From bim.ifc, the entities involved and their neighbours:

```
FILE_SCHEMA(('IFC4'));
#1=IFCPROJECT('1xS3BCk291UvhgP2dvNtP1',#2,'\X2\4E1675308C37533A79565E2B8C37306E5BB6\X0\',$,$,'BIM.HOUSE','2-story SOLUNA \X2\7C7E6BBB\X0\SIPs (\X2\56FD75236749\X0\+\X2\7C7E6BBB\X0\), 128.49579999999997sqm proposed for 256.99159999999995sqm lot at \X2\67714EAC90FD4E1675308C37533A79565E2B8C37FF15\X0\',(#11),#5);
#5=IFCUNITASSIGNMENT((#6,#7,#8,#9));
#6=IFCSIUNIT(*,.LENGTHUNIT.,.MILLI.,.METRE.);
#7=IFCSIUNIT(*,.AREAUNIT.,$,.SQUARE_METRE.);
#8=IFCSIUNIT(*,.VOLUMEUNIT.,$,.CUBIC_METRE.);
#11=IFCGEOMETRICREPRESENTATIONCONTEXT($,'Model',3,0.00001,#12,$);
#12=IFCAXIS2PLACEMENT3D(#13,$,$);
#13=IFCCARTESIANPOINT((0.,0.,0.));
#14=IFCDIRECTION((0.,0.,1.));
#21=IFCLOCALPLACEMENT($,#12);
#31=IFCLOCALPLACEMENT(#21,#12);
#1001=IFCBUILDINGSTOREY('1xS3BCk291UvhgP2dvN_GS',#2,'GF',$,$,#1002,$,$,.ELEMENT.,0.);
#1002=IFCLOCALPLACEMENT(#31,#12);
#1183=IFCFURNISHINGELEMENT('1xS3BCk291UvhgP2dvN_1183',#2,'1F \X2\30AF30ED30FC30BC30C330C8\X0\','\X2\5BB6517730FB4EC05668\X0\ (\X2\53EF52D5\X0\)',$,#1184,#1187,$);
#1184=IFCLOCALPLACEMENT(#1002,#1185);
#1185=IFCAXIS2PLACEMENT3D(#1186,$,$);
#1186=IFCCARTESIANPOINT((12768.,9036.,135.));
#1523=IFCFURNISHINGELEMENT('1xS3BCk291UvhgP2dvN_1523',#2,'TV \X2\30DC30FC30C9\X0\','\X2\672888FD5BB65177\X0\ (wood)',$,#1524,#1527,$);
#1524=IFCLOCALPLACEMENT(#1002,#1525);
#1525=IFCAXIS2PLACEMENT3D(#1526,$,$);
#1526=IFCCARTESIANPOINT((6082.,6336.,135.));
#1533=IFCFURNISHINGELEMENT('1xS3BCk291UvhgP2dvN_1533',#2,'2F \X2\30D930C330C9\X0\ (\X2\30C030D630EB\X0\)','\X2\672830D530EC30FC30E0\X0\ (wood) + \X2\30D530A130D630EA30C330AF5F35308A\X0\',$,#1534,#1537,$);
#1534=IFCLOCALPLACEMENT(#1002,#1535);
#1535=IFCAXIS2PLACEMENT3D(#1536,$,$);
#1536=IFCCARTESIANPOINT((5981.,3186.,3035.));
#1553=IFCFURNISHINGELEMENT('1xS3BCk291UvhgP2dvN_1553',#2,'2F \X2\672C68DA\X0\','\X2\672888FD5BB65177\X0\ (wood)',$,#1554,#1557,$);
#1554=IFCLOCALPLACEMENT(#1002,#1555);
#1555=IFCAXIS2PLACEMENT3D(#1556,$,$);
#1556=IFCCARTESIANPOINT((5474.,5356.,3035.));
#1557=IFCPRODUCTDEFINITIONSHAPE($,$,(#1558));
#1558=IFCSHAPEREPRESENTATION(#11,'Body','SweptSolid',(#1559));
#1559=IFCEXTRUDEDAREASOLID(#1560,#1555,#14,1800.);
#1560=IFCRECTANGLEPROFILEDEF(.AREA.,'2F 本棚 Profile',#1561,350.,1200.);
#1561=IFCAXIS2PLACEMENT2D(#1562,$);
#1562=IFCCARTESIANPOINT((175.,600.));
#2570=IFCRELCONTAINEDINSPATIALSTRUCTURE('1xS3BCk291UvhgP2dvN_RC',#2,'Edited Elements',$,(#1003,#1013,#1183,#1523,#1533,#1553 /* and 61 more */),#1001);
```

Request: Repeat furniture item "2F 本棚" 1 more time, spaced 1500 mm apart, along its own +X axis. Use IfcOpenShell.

```python
import ifcopenshell
import ifcopenshell.api.geometry
import ifcopenshell.api.root
import ifcopenshell.util.element
import ifcopenshell.util.placement
import ifcopenshell.util.unit

model = ifcopenshell.open("bim.ifc")
unit_scale = ifcopenshell.util.unit.calculate_unit_scale(model)


def reuse_history(source, copy):
    """copy_class also copies each property set's owner history, people and application; keep the originals."""
    for rel in copy.IsDefinedBy:
        if rel.is_a("IfcRelDefinesByProperties") and (history := rel.RelatingPropertyDefinition.OwnerHistory):
            rel.RelatingPropertyDefinition.OwnerHistory = source.OwnerHistory
            ifcopenshell.util.element.remove_deep2(model, history)


source = model.by_id(1553)
base = ifcopenshell.util.placement.get_local_placement(source.ObjectPlacement)
step = base[:3, 0] * 1.5 / unit_scale

for i in range(1, 2):
    copy = ifcopenshell.api.root.copy_class(model, product=source)
    copy.Representation = ifcopenshell.util.element.copy_deep(
        model, source.Representation, exclude=["IfcGeometricRepresentationContext", "IfcRepresentationMap"]
    )
    reuse_history(source, copy)
    matrix = base.copy()
    matrix[:3, 3] += i * step
    print("added at", matrix[:3, 3].round(3) + 0.0)
    ifcopenshell.api.geometry.edit_object_placement(model, product=copy, matrix=matrix, is_si=False)

model.write("bim_rev.ifc")
```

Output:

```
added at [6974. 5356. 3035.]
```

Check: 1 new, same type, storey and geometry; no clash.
